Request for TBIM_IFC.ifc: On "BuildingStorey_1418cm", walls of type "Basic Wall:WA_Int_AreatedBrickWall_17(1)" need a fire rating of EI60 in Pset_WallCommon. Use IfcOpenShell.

First a look at what the model holds.

```python
import ifcopenshell
import ifcopenshell.util.element

model = ifcopenshell.open("TBIM_IFC.ifc")
print(model.schema)
storey = next(s for s in model.by_type("IfcBuildingStorey") if s.Name == "BuildingStorey_1418cm")
walls = [e for e in ifcopenshell.util.element.get_decomposition(storey) if e.is_a("IfcWall")]
seen = {}
for e in walls:
    element_type = ifcopenshell.util.element.get_type(e)
    key = (element_type.Name if element_type != e and element_type else None, ifcopenshell.util.element.get_pset(e, "Pset_WallCommon", "FireRating"))
    seen[key] = seen.get(key, 0) + 1
for (name, value), count in sorted(seen.items(), key=str):
    print(count, "x", name, "|", value)
```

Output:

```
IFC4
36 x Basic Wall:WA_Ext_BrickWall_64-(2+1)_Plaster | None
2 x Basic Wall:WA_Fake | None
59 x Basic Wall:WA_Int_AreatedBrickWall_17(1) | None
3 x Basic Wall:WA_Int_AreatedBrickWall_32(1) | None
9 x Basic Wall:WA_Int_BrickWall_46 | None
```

```python
import ifcopenshell
import ifcopenshell.api.pset
import ifcopenshell.util.element

model = ifcopenshell.open("TBIM_IFC.ifc")

storey = next(s for s in model.by_type("IfcBuildingStorey") if s.Name == "BuildingStorey_1418cm")
walls = [e for e in ifcopenshell.util.element.get_decomposition(storey) if e.is_a("IfcWall")]

count = 0
for e in walls:
    element_type = ifcopenshell.util.element.get_type(e)
    if element_type in (None, e) or element_type.Name != "Basic Wall:WA_Int_AreatedBrickWall_17(1)":
        continue
    # add_pset returns the element's existing set when there is one.
    pset = ifcopenshell.api.pset.add_pset(model, product=e, name="Pset_WallCommon")
    ifcopenshell.api.pset.edit_pset(model, pset=pset, properties={"FireRating": "EI60"})
    count += 1

print(count, "walls updated")

model.write("TBIM_IFC_v2.ifc")
```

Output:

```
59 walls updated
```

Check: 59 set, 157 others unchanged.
